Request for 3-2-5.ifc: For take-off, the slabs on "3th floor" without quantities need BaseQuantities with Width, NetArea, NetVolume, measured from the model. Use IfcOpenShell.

First a look at what the model holds.

```python
import ifcopenshell
import ifcopenshell.util.element
import ifcopenshell.util.unit

model = ifcopenshell.open("3-2-5.ifc")
print(model.schema)
for unit_type in ("LENGTHUNIT", "AREAUNIT", "VOLUMEUNIT"):
    print(unit_type, ifcopenshell.util.unit.calculate_unit_scale(model, unit_type))
storey = next(s for s in model.by_type("IfcBuildingStorey") if s.Name == "3th floor")
slabs = [e for e in ifcopenshell.util.element.get_decomposition(storey) if e.is_a("IfcSlab")]
for e in sorted(slabs, key=lambda e: e.id()):
    print(e.id(), e.is_a(), e.Name, list(ifcopenshell.util.element.get_psets(e, qtos_only=True)), sep=" | ")
```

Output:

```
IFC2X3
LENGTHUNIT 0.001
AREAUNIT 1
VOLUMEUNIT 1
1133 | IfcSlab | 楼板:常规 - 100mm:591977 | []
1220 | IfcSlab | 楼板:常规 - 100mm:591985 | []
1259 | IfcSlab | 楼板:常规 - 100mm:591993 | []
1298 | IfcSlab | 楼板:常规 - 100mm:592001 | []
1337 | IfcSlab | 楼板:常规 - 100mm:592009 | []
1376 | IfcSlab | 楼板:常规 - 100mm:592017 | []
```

```python
import ifcopenshell
import ifcopenshell.api.pset
import ifcopenshell.geom
import ifcopenshell.util.element
import ifcopenshell.util.shape
import ifcopenshell.util.unit

model = ifcopenshell.open("3-2-5.ifc")
unit_scale = ifcopenshell.util.unit.calculate_unit_scale(model)
area_scale = ifcopenshell.util.unit.calculate_unit_scale(model, "AREAUNIT")
volume_scale = ifcopenshell.util.unit.calculate_unit_scale(model, "VOLUMEUNIT")
settings = ifcopenshell.geom.settings()

storey = next(s for s in model.by_type("IfcBuildingStorey") if s.Name == "3th floor")
slabs = [e for e in ifcopenshell.util.element.get_decomposition(storey) if e.is_a("IfcSlab")]

for e in sorted(slabs, key=lambda e: e.id()):
    if ifcopenshell.util.element.get_psets(e, qtos_only=True, should_inherit=False):
        continue
    # Geometry comes back in metres, in the element's own axes.
    shape = ifcopenshell.geom.create_shape(settings, e)
    values = {
        "Width": ifcopenshell.util.shape.get_z(shape.geometry) / unit_scale,
        "NetArea": ifcopenshell.util.shape.get_footprint_area(shape.geometry) / area_scale,
        "NetVolume": ifcopenshell.util.shape.get_volume(shape.geometry) / volume_scale,
    }
    qto = ifcopenshell.api.pset.add_qto(model, product=e, name="BaseQuantities")
    ifcopenshell.api.pset.edit_qto(model, qto=qto, properties=values)
    print(e.id(), {k: round(v, 3) for k, v in values.items()})

model.write("3-2-5_v2.ifc")
```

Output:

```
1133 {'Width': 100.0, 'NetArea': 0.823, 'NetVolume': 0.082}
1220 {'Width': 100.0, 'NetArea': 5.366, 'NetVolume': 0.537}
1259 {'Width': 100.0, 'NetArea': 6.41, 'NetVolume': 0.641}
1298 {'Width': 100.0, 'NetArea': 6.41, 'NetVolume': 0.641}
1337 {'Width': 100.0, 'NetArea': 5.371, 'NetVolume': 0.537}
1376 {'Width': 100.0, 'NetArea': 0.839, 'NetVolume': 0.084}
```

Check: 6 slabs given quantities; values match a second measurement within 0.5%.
